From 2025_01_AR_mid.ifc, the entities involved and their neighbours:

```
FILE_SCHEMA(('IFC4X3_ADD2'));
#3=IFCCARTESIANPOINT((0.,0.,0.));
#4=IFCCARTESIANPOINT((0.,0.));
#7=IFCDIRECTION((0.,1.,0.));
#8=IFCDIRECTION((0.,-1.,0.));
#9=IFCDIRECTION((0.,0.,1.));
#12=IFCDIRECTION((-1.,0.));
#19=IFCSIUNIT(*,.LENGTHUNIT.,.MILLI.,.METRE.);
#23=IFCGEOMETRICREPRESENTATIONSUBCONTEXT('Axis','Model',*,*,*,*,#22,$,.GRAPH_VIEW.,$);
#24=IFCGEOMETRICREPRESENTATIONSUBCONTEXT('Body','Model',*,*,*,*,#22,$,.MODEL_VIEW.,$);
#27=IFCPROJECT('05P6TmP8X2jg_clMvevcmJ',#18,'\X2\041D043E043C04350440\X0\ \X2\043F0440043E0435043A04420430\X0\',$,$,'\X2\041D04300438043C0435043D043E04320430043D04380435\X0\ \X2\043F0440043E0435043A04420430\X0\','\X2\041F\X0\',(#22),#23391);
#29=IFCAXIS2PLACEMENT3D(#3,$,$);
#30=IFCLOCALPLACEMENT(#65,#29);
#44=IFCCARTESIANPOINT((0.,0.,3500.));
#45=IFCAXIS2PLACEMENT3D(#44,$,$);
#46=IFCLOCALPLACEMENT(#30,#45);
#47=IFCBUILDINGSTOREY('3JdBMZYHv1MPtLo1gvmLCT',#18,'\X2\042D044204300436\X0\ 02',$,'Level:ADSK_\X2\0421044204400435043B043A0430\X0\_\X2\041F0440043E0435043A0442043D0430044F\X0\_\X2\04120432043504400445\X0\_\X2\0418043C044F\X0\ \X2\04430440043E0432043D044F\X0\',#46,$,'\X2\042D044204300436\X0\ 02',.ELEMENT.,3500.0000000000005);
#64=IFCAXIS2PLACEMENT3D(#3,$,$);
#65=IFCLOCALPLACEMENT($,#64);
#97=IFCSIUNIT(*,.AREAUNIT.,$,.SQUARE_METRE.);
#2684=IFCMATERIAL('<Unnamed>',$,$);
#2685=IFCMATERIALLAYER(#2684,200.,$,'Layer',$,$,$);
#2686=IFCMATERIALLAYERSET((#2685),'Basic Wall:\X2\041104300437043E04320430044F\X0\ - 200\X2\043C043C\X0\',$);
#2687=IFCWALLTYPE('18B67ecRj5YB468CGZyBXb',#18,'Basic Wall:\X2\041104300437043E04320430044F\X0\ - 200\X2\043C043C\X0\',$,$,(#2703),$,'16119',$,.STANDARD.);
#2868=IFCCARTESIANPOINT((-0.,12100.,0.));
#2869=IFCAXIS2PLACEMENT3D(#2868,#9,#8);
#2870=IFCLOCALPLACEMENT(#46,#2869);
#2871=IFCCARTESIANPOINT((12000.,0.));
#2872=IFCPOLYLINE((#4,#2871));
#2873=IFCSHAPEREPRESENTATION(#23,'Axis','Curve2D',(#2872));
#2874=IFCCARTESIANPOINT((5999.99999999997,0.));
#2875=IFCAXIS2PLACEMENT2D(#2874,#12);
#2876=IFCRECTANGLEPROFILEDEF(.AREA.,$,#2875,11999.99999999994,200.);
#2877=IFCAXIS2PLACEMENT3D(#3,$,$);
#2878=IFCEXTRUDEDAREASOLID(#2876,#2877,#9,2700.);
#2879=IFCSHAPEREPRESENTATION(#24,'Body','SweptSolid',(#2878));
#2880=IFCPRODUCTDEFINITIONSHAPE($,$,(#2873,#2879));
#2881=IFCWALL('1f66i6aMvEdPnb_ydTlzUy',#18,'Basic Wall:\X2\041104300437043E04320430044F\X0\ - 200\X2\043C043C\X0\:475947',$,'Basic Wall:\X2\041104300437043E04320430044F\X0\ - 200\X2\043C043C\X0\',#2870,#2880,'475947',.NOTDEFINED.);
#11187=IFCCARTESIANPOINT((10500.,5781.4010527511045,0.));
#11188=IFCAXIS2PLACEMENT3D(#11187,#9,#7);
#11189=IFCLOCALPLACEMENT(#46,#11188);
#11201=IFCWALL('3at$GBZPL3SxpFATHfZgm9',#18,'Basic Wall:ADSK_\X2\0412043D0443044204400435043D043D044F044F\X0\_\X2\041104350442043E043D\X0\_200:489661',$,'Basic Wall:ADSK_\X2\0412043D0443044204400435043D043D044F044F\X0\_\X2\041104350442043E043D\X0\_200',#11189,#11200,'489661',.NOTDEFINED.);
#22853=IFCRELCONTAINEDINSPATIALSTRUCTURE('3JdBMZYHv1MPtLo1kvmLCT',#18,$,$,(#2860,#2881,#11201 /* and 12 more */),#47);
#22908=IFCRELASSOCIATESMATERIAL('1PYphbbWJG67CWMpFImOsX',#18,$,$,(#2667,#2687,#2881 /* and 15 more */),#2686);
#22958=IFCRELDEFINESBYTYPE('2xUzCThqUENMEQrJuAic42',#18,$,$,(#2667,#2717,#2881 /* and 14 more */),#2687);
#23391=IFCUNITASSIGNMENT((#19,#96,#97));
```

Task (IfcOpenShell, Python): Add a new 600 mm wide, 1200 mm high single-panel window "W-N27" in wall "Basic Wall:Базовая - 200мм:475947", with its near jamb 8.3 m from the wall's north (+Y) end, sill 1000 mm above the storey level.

```python
import numpy as np
import ifcopenshell
import ifcopenshell.api.feature
import ifcopenshell.api.geometry
import ifcopenshell.api.root
import ifcopenshell.api.spatial
import ifcopenshell.geom
import ifcopenshell.util.element
import ifcopenshell.util.placement
import ifcopenshell.util.representation
import ifcopenshell.util.shape
import ifcopenshell.util.unit

model = ifcopenshell.open("2025_01_AR_mid.ifc")
unit_scale = ifcopenshell.util.unit.calculate_unit_scale(model)
settings = ifcopenshell.geom.settings()


def volume(element):
    """Net volume in cubic metres, openings subtracted."""
    shape = ifcopenshell.geom.create_shape(settings, element)
    return ifcopenshell.util.shape.get_volume(shape.geometry)


wall = model.by_id(2881)
storey = ifcopenshell.util.element.get_container(wall, ifc_class="IfcBuildingStorey")
context = ifcopenshell.util.representation.get_context(model, "Model", "Body", "MODEL_VIEW")
before = volume(wall)

width, height, from_end, sill = 0.6, 1.2, 8.3, 1  # metres

# The wall runs along its own X axis, and the end named is its -X end.
wall_shape = ifcopenshell.geom.create_shape(settings, wall)
x, y, z = ifcopenshell.util.shape.get_vertices(wall_shape.geometry).T
start = x.min() + from_end
face, thickness = float(y.min()), float(y.max() - y.min())
wall_matrix = ifcopenshell.util.placement.get_local_placement(wall.ObjectPlacement)
level = ifcopenshell.util.placement.get_local_placement(storey.ObjectPlacement)[2, 3]


def in_wall(x, y):
    """Placement at x, y metres in the wall's axes, at sill height."""
    matrix = wall_matrix.copy()
    matrix[:, 3] = wall_matrix @ np.array([x / unit_scale, y / unit_scale, 0.0, 1.0])
    matrix[2, 3] = level + sill / unit_scale
    return matrix


# Opening: a box that overshoots both wall faces by 50 mm.
opening = ifcopenshell.api.root.create_entity(model, ifc_class="IfcOpeningElement", predefined_type="OPENING")
box = ifcopenshell.api.geometry.add_wall_representation(
    model, context=context, length=width, height=height, thickness=thickness + 0.1
)
ifcopenshell.api.geometry.assign_representation(model, product=opening, representation=box)
ifcopenshell.api.geometry.edit_object_placement(model, product=opening, matrix=in_wall(start, face - 0.05), is_si=False)
ifcopenshell.api.feature.add_feature(model, feature=opening, element=wall)

window = ifcopenshell.api.root.create_entity(model, ifc_class="IfcWindow", name="W-N27", predefined_type="WINDOW")
window.OverallWidth, window.OverallHeight = width / unit_scale, height / unit_scale
window.PartitioningType = "SINGLE_PANEL"
body = ifcopenshell.api.geometry.add_window_representation(
    model,
    context=context,
    overall_width=window.OverallWidth,
    overall_height=window.OverallHeight,
    partition_type="SINGLE_PANEL",
)
ifcopenshell.api.geometry.assign_representation(model, product=window, representation=body)
ifcopenshell.api.spatial.assign_container(model, products=[window], relating_structure=storey)
ifcopenshell.api.feature.add_filling(model, opening=opening, element=window)

# Centre the window in the wall's thickness.
ifcopenshell.api.geometry.edit_object_placement(model, product=window, matrix=in_wall(start, face), is_si=False)
window_shape = ifcopenshell.geom.create_shape(settings, window)
depth = ifcopenshell.util.shape.get_vertices(window_shape.geometry)[:, 1]
offset = face + thickness / 2 - (depth.min() + depth.max()) / 2
ifcopenshell.api.geometry.edit_object_placement(model, product=window, matrix=in_wall(start, offset), is_si=False)

after = volume(wall)

print(f"wall volume {before:.3f} -> {after:.3f} m3")

model.write("2025_01_AR_mid_edited.ifc")
```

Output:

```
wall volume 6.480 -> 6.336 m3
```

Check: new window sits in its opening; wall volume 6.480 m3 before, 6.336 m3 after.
